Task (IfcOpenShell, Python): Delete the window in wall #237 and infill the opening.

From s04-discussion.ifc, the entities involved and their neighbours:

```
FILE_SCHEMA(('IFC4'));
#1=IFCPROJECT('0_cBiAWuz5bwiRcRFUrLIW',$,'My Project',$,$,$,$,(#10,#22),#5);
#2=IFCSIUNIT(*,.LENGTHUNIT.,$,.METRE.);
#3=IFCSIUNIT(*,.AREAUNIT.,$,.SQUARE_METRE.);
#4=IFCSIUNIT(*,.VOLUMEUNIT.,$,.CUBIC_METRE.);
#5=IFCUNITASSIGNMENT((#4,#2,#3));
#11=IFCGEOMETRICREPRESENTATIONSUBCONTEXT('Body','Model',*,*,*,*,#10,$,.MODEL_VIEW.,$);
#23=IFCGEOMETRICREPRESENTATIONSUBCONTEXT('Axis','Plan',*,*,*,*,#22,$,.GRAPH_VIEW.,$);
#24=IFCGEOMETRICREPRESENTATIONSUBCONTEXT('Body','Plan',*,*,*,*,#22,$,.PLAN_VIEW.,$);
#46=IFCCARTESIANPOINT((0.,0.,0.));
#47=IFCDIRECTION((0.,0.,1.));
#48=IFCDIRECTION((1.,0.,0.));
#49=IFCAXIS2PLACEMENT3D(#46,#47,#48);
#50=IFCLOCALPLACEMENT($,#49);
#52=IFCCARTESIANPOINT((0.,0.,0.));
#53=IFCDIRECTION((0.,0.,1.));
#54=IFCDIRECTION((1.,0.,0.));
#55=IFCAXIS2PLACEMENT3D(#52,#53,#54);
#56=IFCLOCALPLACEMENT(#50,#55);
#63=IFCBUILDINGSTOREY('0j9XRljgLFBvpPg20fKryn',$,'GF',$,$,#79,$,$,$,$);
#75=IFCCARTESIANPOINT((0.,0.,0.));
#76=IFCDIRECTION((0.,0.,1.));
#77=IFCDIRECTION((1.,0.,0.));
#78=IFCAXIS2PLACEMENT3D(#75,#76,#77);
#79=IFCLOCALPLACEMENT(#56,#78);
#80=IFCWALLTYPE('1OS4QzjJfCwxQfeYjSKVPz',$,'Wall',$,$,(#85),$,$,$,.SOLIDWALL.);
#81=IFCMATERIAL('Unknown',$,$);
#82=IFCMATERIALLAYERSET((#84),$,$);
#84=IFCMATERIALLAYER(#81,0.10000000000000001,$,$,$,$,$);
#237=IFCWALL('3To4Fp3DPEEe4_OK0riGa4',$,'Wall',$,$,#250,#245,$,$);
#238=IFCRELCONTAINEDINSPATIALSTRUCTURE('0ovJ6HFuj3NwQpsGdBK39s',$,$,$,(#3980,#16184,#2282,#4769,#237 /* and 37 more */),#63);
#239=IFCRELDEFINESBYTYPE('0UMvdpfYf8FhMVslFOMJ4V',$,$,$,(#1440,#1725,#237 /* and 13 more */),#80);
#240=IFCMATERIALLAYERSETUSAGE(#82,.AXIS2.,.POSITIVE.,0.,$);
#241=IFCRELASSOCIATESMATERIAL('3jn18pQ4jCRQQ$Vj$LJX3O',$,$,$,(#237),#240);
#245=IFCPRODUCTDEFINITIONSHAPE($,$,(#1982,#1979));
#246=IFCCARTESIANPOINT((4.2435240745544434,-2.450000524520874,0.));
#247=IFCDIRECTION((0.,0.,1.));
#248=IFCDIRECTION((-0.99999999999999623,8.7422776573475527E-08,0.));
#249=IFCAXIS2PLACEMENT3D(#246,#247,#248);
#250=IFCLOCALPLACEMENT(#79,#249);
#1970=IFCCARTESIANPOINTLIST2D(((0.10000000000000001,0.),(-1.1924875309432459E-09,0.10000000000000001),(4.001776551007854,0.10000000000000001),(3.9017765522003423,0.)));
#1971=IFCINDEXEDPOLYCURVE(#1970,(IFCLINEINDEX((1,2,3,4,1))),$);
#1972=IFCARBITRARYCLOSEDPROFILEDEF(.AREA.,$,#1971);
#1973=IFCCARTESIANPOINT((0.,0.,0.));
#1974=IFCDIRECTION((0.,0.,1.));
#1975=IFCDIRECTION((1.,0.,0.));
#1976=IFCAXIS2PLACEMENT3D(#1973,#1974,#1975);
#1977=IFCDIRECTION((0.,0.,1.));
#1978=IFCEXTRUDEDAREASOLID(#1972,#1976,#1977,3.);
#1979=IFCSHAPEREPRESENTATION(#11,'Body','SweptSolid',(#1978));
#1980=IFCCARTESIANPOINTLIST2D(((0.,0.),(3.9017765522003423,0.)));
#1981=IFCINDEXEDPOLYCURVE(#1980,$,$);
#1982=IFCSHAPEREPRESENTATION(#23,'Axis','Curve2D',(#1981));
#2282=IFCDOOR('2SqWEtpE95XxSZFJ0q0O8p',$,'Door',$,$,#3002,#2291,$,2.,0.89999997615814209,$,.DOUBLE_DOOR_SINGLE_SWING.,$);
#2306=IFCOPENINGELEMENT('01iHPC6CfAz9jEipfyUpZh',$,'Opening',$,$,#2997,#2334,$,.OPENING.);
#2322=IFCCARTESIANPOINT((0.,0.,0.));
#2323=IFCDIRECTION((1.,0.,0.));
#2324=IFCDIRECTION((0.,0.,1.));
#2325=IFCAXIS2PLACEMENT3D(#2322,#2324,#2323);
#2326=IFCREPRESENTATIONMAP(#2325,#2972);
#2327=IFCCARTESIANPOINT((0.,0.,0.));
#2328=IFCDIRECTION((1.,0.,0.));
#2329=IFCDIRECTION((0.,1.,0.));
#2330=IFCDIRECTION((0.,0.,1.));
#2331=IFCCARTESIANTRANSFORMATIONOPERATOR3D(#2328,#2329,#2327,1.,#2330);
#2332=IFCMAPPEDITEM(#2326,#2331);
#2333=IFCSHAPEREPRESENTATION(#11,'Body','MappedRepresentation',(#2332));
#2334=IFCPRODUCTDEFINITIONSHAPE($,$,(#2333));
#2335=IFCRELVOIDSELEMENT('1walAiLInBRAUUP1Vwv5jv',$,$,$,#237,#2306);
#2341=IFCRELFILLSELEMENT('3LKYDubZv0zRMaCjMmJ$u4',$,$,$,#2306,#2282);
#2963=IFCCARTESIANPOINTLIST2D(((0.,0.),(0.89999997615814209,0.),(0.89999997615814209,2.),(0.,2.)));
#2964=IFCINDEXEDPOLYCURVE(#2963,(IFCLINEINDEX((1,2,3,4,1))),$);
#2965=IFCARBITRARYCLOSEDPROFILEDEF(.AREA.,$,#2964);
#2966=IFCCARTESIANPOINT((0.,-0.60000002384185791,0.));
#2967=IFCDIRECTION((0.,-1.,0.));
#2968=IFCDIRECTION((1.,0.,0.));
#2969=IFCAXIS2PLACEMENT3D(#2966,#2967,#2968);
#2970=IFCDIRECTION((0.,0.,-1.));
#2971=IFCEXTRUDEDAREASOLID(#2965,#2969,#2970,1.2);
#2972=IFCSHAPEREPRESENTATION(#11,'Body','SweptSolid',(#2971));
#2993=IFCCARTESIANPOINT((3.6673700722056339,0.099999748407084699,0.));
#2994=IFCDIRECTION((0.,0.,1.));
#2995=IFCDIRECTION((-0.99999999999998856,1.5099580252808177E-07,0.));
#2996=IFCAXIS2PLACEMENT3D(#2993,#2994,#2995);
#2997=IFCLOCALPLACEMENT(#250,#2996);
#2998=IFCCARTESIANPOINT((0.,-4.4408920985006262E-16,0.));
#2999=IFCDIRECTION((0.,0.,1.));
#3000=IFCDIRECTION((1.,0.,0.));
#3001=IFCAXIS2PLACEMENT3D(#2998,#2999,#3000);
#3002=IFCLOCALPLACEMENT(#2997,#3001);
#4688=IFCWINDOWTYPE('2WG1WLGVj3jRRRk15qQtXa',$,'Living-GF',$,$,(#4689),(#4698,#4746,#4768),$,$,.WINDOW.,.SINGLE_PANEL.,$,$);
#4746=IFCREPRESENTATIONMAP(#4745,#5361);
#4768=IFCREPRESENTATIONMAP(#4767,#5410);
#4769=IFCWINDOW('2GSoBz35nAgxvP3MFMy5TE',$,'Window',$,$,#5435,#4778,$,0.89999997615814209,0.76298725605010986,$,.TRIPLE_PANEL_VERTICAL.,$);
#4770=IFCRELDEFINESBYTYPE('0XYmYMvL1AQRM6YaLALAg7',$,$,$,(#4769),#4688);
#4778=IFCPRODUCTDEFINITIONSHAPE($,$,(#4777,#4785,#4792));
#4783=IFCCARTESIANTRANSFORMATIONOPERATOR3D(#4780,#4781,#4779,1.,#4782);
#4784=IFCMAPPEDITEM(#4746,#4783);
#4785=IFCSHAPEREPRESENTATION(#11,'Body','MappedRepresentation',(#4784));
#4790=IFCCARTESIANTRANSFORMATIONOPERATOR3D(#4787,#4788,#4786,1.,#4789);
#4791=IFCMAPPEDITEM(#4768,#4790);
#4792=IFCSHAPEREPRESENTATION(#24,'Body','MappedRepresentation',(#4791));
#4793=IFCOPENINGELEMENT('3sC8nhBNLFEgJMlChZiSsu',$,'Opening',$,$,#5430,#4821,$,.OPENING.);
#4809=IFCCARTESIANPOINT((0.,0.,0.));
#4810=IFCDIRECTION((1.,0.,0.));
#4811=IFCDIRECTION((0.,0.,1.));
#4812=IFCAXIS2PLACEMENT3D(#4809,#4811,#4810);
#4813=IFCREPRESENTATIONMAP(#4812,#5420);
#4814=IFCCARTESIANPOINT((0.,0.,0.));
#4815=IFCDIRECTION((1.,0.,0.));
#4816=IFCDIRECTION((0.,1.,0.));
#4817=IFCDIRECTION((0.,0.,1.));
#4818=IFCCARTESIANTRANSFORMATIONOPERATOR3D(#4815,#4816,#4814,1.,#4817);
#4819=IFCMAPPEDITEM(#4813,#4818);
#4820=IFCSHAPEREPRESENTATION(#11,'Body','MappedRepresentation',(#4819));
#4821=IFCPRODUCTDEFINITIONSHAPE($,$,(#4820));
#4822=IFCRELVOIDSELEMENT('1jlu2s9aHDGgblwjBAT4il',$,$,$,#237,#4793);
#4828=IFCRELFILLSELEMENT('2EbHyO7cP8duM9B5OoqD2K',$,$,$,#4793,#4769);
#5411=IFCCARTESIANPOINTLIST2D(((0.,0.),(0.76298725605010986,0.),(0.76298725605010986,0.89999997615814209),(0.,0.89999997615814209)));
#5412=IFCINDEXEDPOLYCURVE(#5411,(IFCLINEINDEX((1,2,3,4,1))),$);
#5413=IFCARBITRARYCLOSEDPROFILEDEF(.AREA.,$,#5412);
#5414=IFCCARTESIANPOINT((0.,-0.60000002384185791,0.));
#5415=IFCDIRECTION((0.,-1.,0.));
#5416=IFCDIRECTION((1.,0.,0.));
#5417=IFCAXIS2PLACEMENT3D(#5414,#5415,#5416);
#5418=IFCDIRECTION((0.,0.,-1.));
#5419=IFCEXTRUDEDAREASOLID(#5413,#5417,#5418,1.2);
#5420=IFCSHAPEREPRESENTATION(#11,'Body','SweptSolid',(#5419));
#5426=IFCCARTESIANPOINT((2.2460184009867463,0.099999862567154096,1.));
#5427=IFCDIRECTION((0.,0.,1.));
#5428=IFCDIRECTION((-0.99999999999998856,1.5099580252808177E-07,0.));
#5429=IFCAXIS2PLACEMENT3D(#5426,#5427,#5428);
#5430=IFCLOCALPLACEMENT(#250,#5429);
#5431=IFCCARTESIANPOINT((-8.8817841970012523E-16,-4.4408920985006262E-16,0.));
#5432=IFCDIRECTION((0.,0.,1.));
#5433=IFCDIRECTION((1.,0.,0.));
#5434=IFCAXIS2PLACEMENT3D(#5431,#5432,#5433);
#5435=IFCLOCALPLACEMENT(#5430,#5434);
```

```python
import ifcopenshell
import ifcopenshell.api.feature
import ifcopenshell.api.root
import ifcopenshell.geom
import ifcopenshell.util.shape

model = ifcopenshell.open("s04-discussion.ifc")
settings = ifcopenshell.geom.settings()


def volume(element):
    """Net volume in cubic metres, openings subtracted."""
    shape = ifcopenshell.geom.create_shape(settings, element)
    return ifcopenshell.util.shape.get_volume(shape.geometry)


window = model.by_id(4769)
opening = window.FillsVoids[0].RelatingOpeningElement
wall = opening.VoidsElements[0].RelatingBuildingElement
before = volume(wall)

ifcopenshell.api.root.remove_product(model, product=window)
ifcopenshell.api.feature.remove_feature(model, feature=opening)

after = volume(wall)

print(f"wall volume {before:.3f} -> {after:.3f} m3")

model.write("s04-discussion_rev.ifc")
```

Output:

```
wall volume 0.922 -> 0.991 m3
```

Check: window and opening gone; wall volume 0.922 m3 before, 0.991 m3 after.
